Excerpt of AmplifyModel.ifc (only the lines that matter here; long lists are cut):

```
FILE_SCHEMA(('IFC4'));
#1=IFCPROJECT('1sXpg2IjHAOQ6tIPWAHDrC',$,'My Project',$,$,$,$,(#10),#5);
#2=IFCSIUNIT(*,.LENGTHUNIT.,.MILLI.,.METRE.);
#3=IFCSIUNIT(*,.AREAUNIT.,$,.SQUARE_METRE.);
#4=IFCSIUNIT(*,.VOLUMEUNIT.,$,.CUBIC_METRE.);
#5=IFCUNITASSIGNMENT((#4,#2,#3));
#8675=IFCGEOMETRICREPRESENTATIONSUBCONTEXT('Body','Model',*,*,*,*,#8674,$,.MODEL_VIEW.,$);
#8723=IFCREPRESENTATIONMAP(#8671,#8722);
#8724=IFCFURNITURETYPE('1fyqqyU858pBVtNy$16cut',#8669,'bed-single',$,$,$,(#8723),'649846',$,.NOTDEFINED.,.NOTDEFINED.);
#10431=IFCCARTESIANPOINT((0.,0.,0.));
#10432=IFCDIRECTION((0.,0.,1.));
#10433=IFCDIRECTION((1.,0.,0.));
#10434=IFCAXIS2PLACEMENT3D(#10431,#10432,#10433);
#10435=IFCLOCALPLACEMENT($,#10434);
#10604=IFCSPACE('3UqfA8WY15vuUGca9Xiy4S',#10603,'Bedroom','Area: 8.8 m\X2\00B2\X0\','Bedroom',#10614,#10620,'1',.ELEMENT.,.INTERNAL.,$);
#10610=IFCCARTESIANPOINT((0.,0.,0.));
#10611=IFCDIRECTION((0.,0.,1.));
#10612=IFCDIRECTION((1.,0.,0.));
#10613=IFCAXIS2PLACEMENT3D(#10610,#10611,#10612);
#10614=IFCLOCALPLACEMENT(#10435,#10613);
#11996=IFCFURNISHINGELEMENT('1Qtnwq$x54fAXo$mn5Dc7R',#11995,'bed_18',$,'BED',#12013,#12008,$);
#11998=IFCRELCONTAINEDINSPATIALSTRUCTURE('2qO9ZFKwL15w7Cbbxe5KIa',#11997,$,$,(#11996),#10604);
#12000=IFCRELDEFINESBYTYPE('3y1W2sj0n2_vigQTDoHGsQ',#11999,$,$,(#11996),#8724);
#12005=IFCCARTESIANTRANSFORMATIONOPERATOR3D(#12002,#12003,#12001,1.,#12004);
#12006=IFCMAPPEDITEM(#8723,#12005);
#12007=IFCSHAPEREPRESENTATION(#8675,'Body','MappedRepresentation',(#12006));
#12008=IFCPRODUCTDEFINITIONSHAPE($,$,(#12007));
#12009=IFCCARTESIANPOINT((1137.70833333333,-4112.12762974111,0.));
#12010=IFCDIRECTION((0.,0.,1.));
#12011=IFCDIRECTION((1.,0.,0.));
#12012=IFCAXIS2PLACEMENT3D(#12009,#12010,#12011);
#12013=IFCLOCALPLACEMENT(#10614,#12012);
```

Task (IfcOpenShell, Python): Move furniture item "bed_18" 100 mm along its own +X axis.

```python
import ifcopenshell
import ifcopenshell.api.geometry
import ifcopenshell.util.placement
import ifcopenshell.util.unit

model = ifcopenshell.open("AmplifyModel.ifc")
unit_scale = ifcopenshell.util.unit.calculate_unit_scale(model)

item = model.by_guid("1Qtnwq$x54fAXo$mn5Dc7R")
matrix = ifcopenshell.util.placement.get_local_placement(item.ObjectPlacement)
matrix[:3, 3] += matrix[:3, 0] * 0.1 / unit_scale
ifcopenshell.api.geometry.edit_object_placement(model, product=item, matrix=matrix, is_si=False)

print(ifcopenshell.util.placement.get_local_placement(item.ObjectPlacement).round(3) + 0.0)

model.write("AmplifyModel_v2.ifc")
```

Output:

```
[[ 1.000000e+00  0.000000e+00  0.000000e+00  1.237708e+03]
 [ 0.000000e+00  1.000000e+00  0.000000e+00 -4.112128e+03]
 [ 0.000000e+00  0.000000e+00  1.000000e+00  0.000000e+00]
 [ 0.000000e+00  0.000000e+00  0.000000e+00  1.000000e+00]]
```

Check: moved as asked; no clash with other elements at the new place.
